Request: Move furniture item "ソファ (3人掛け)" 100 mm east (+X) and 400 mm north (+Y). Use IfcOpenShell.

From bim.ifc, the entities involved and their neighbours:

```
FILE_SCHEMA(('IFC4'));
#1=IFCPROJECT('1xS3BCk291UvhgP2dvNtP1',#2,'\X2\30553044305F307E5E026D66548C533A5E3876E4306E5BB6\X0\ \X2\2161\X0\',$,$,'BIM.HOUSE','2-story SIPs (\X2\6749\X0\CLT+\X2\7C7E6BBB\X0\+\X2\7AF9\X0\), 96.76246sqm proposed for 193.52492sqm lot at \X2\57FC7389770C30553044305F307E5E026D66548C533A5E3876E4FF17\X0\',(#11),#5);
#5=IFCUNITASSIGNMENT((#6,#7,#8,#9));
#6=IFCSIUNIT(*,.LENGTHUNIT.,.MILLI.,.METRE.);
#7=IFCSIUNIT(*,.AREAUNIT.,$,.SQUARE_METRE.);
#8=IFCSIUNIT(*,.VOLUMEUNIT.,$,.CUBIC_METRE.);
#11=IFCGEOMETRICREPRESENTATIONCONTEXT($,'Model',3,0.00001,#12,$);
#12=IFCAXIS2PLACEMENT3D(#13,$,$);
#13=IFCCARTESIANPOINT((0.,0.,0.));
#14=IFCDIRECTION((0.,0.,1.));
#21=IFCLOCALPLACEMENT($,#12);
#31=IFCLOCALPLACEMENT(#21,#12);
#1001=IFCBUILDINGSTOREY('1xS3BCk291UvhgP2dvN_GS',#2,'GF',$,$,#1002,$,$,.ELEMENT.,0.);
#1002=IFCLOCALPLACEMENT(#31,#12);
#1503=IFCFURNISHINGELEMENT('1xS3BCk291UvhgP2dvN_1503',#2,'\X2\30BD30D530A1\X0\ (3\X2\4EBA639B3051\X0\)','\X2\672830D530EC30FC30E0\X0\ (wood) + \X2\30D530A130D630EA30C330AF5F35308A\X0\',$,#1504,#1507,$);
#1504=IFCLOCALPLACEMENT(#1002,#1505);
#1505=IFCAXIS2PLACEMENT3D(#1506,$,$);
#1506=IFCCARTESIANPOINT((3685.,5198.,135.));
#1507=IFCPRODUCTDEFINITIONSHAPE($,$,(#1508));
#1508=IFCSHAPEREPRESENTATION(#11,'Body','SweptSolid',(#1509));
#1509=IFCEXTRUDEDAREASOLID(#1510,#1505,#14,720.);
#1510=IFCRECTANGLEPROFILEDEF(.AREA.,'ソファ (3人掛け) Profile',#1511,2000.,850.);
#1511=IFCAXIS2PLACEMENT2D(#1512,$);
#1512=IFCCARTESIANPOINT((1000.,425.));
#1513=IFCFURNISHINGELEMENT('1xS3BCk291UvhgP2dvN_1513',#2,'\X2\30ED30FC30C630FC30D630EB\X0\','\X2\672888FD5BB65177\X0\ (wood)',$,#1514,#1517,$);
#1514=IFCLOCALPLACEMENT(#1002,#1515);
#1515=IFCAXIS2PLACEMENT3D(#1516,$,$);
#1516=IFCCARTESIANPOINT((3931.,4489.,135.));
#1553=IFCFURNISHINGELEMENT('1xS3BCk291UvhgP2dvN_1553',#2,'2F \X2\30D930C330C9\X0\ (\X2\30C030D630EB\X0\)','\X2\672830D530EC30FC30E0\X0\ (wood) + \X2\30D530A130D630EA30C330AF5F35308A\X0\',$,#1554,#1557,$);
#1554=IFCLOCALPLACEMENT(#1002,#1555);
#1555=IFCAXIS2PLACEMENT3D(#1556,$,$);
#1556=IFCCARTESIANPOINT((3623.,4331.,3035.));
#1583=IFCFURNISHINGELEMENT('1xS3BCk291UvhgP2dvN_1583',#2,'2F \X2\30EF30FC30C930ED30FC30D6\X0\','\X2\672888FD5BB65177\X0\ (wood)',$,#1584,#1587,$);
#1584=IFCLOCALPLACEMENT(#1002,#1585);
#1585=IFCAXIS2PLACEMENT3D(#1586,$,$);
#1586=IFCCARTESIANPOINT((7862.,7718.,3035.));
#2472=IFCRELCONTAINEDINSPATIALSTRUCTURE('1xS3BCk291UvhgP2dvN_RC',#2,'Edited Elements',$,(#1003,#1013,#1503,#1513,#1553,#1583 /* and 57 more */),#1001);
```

```python
import ifcopenshell
import ifcopenshell.api.geometry
import ifcopenshell.util.placement

model = ifcopenshell.open("bim.ifc")

item = model.by_id(1503)
matrix = ifcopenshell.util.placement.get_local_placement(item.ObjectPlacement)
matrix[0, 3] += 100.0
matrix[1, 3] += 400.0
ifcopenshell.api.geometry.edit_object_placement(model, product=item, matrix=matrix, is_si=False)

print(ifcopenshell.util.placement.get_local_placement(item.ObjectPlacement).round(3) + 0.0)

model.write("bim_edited.ifc")
```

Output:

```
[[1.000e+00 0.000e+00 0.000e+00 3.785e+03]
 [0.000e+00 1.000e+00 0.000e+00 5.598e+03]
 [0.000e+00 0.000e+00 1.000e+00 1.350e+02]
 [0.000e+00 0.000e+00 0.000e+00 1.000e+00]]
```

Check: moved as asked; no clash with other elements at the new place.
